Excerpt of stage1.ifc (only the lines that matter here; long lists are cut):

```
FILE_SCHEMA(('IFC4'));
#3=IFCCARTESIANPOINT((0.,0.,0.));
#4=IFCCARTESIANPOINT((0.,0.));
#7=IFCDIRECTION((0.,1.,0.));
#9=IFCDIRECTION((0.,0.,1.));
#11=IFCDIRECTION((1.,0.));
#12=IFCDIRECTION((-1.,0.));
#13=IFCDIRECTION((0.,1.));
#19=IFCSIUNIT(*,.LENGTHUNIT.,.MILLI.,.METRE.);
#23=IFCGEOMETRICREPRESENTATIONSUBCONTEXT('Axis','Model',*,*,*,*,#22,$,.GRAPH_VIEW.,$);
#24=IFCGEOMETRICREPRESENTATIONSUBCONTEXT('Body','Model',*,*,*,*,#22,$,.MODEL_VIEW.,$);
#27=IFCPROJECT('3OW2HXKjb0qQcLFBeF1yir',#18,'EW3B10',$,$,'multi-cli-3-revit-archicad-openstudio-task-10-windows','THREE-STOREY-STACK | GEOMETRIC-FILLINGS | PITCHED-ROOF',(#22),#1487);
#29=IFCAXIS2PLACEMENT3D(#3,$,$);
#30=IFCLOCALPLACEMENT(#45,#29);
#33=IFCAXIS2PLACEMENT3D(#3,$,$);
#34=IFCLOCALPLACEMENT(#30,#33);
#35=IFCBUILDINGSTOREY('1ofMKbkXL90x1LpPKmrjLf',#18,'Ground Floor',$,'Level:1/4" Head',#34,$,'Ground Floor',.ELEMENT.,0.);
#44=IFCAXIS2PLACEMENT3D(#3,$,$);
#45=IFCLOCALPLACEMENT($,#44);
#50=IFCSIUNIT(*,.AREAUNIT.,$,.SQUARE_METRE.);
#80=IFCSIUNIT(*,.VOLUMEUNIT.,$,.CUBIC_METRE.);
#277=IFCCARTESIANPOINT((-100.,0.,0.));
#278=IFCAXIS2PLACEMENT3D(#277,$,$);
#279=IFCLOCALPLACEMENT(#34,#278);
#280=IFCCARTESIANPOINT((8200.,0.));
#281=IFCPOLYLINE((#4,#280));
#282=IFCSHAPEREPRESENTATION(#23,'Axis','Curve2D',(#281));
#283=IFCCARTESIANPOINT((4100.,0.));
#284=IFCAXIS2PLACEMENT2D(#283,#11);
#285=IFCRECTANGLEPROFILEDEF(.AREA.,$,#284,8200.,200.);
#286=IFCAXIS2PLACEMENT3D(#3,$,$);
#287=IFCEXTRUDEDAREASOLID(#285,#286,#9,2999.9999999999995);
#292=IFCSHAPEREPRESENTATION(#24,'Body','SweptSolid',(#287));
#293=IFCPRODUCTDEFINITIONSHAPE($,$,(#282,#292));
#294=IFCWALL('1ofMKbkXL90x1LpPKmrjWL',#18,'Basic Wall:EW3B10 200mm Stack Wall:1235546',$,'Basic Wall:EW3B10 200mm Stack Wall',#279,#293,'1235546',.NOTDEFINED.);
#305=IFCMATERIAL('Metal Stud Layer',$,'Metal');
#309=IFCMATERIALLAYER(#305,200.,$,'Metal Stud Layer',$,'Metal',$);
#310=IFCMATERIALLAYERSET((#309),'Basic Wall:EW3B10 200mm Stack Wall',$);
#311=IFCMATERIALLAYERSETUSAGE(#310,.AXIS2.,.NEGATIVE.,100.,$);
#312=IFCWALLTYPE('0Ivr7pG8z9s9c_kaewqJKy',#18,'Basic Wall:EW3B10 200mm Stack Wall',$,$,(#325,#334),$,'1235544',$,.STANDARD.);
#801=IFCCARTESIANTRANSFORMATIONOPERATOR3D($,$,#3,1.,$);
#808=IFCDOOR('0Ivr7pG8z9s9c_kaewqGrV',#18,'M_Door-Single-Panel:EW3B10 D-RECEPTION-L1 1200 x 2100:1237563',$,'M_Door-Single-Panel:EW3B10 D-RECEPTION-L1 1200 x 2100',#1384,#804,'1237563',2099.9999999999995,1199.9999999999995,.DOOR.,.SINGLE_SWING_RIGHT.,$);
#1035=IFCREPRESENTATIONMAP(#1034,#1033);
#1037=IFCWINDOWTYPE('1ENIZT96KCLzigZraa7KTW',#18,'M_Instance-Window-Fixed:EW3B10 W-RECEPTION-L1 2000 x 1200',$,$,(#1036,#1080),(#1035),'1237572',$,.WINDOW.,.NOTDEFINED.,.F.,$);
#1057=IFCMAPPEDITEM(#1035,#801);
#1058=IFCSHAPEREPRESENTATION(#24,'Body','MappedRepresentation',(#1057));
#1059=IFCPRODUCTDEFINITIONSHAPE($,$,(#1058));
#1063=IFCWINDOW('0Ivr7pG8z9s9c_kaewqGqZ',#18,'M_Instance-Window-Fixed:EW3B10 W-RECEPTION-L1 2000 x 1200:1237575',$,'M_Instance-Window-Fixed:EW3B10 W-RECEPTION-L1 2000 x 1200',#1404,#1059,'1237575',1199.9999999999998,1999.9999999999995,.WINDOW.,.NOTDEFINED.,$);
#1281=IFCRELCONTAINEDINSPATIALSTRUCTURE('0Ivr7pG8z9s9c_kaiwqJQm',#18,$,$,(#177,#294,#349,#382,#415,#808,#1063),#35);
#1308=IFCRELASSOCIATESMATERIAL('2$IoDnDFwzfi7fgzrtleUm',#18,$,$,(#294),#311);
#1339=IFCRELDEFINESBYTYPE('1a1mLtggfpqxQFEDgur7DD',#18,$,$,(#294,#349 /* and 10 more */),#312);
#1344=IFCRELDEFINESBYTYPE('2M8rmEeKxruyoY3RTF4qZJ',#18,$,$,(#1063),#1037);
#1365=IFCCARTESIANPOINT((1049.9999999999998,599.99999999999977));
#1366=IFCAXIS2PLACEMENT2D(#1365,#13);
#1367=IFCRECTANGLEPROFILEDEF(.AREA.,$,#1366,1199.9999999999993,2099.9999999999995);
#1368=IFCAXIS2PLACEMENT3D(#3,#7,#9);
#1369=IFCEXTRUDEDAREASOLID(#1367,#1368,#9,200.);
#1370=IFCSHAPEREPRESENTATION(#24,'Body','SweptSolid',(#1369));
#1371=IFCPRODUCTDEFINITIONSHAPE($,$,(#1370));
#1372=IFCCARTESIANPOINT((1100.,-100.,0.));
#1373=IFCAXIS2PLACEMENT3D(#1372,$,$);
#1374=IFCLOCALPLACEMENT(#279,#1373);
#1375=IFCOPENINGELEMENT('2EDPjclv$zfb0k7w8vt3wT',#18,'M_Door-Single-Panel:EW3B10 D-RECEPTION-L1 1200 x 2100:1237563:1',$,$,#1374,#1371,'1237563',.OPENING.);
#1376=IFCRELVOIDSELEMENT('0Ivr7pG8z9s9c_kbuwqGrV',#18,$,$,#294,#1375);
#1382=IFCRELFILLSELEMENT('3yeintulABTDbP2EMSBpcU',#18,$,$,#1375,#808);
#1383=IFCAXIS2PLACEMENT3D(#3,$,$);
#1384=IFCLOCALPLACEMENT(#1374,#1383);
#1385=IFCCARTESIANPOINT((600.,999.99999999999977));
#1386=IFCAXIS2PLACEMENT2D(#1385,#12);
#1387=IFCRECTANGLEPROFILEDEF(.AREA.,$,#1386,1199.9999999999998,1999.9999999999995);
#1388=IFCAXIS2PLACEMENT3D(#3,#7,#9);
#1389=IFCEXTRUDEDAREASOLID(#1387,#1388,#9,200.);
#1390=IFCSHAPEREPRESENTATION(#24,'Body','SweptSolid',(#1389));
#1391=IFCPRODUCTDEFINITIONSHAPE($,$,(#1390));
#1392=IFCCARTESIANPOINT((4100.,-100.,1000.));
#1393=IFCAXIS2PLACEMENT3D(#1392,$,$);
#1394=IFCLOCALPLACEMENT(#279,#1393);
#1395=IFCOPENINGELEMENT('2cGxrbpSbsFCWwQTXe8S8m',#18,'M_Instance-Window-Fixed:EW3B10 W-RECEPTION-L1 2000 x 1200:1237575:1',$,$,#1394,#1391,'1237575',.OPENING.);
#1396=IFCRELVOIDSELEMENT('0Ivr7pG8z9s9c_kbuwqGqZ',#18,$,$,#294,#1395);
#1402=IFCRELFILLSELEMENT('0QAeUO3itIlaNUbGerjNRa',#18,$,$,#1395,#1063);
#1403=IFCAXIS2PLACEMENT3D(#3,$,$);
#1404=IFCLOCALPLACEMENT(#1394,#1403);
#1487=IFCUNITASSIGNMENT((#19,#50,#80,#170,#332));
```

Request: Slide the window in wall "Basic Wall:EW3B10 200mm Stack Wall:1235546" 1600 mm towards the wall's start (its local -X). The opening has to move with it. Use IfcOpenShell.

```python
import ifcopenshell
import ifcopenshell.api.geometry
import ifcopenshell.util.placement

model = ifcopenshell.open("stage1.ifc")

window = model.by_guid("0Ivr7pG8z9s9c_kaewqGqZ")
opening = window.FillsVoids[0].RelatingOpeningElement
wall = opening.VoidsElements[0].RelatingBuildingElement

wall_matrix = ifcopenshell.util.placement.get_local_placement(wall.ObjectPlacement)
shift = wall_matrix[:3, 0] * -1600.0
before = ifcopenshell.util.placement.get_local_placement(window.ObjectPlacement)[:3, 3].copy()

# The window is placed relative to its opening, so it follows when the opening moves.
matrix = ifcopenshell.util.placement.get_local_placement(opening.ObjectPlacement)
matrix[:3, 3] += shift
ifcopenshell.api.geometry.edit_object_placement(
    model, product=opening, matrix=matrix, is_si=False, should_transform_children=True
)

after = ifcopenshell.util.placement.get_local_placement(window.ObjectPlacement)[:3, 3]
print("window moved by", (after - before).round(3) + 0.0)

model.write("stage1-out.ifc")
```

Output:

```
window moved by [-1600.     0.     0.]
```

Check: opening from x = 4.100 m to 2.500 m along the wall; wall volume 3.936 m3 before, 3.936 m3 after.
